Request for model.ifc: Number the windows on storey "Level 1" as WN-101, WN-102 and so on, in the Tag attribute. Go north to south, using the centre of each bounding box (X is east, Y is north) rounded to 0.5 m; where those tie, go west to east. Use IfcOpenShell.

First a look at what the model holds.

```python
import ifcopenshell
import ifcopenshell.util.element
import ifcopenshell.util.placement

model = ifcopenshell.open("model.ifc")
print(model.schema)
storey = next(s for s in model.by_type("IfcBuildingStorey") if s.Name == "Level 1")
windows = [e for e in ifcopenshell.util.element.get_decomposition(storey) if e.is_a("IfcWindow")]
for e in sorted(windows, key=lambda e: e.id()):
    origin = ifcopenshell.util.placement.get_local_placement(e.ObjectPlacement)[:3, 3]
    print(e.id(), e.Tag, e.Name, origin.round(2) + 0.0, sep=" | ")
```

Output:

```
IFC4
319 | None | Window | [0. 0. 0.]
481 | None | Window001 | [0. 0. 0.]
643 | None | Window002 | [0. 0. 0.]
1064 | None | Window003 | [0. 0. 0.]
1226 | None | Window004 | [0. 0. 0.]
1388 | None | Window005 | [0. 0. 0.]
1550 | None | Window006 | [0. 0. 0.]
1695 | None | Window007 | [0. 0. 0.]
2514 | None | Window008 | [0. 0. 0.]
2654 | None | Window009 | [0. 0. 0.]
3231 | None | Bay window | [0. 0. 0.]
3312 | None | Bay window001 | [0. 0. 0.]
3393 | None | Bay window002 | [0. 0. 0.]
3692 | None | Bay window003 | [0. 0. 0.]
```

```python
import ifcopenshell
import ifcopenshell.geom
import ifcopenshell.util.element
import ifcopenshell.util.shape

model = ifcopenshell.open("model.ifc")
settings = ifcopenshell.geom.settings()
settings.set("use-world-coords", True)


def centre(element):
    shape = ifcopenshell.geom.create_shape(settings, element)
    return ifcopenshell.util.shape.get_bbox_centroid(shape.geometry)


storey = next(s for s in model.by_type("IfcBuildingStorey") if s.Name == "Level 1")
windows = [e for e in ifcopenshell.util.element.get_decomposition(storey) if e.is_a("IfcWindow")]

# Insertion points can sit at a corner or the storey origin, so sort by the geometry (in metres).
centres = {e: centre(e) for e in windows}
windows.sort(key=lambda e: (-round(centres[e][1] / 0.5), centres[e][0]))

for i, e in enumerate(windows, start=1):
    number = f"WN-1{i:02d}"
    e.Tag = number
    print(e.id(), number)

model.write("model_updated.ifc")
```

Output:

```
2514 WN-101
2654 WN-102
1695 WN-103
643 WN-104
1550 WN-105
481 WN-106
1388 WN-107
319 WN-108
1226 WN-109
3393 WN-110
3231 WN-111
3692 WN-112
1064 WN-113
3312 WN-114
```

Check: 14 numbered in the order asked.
